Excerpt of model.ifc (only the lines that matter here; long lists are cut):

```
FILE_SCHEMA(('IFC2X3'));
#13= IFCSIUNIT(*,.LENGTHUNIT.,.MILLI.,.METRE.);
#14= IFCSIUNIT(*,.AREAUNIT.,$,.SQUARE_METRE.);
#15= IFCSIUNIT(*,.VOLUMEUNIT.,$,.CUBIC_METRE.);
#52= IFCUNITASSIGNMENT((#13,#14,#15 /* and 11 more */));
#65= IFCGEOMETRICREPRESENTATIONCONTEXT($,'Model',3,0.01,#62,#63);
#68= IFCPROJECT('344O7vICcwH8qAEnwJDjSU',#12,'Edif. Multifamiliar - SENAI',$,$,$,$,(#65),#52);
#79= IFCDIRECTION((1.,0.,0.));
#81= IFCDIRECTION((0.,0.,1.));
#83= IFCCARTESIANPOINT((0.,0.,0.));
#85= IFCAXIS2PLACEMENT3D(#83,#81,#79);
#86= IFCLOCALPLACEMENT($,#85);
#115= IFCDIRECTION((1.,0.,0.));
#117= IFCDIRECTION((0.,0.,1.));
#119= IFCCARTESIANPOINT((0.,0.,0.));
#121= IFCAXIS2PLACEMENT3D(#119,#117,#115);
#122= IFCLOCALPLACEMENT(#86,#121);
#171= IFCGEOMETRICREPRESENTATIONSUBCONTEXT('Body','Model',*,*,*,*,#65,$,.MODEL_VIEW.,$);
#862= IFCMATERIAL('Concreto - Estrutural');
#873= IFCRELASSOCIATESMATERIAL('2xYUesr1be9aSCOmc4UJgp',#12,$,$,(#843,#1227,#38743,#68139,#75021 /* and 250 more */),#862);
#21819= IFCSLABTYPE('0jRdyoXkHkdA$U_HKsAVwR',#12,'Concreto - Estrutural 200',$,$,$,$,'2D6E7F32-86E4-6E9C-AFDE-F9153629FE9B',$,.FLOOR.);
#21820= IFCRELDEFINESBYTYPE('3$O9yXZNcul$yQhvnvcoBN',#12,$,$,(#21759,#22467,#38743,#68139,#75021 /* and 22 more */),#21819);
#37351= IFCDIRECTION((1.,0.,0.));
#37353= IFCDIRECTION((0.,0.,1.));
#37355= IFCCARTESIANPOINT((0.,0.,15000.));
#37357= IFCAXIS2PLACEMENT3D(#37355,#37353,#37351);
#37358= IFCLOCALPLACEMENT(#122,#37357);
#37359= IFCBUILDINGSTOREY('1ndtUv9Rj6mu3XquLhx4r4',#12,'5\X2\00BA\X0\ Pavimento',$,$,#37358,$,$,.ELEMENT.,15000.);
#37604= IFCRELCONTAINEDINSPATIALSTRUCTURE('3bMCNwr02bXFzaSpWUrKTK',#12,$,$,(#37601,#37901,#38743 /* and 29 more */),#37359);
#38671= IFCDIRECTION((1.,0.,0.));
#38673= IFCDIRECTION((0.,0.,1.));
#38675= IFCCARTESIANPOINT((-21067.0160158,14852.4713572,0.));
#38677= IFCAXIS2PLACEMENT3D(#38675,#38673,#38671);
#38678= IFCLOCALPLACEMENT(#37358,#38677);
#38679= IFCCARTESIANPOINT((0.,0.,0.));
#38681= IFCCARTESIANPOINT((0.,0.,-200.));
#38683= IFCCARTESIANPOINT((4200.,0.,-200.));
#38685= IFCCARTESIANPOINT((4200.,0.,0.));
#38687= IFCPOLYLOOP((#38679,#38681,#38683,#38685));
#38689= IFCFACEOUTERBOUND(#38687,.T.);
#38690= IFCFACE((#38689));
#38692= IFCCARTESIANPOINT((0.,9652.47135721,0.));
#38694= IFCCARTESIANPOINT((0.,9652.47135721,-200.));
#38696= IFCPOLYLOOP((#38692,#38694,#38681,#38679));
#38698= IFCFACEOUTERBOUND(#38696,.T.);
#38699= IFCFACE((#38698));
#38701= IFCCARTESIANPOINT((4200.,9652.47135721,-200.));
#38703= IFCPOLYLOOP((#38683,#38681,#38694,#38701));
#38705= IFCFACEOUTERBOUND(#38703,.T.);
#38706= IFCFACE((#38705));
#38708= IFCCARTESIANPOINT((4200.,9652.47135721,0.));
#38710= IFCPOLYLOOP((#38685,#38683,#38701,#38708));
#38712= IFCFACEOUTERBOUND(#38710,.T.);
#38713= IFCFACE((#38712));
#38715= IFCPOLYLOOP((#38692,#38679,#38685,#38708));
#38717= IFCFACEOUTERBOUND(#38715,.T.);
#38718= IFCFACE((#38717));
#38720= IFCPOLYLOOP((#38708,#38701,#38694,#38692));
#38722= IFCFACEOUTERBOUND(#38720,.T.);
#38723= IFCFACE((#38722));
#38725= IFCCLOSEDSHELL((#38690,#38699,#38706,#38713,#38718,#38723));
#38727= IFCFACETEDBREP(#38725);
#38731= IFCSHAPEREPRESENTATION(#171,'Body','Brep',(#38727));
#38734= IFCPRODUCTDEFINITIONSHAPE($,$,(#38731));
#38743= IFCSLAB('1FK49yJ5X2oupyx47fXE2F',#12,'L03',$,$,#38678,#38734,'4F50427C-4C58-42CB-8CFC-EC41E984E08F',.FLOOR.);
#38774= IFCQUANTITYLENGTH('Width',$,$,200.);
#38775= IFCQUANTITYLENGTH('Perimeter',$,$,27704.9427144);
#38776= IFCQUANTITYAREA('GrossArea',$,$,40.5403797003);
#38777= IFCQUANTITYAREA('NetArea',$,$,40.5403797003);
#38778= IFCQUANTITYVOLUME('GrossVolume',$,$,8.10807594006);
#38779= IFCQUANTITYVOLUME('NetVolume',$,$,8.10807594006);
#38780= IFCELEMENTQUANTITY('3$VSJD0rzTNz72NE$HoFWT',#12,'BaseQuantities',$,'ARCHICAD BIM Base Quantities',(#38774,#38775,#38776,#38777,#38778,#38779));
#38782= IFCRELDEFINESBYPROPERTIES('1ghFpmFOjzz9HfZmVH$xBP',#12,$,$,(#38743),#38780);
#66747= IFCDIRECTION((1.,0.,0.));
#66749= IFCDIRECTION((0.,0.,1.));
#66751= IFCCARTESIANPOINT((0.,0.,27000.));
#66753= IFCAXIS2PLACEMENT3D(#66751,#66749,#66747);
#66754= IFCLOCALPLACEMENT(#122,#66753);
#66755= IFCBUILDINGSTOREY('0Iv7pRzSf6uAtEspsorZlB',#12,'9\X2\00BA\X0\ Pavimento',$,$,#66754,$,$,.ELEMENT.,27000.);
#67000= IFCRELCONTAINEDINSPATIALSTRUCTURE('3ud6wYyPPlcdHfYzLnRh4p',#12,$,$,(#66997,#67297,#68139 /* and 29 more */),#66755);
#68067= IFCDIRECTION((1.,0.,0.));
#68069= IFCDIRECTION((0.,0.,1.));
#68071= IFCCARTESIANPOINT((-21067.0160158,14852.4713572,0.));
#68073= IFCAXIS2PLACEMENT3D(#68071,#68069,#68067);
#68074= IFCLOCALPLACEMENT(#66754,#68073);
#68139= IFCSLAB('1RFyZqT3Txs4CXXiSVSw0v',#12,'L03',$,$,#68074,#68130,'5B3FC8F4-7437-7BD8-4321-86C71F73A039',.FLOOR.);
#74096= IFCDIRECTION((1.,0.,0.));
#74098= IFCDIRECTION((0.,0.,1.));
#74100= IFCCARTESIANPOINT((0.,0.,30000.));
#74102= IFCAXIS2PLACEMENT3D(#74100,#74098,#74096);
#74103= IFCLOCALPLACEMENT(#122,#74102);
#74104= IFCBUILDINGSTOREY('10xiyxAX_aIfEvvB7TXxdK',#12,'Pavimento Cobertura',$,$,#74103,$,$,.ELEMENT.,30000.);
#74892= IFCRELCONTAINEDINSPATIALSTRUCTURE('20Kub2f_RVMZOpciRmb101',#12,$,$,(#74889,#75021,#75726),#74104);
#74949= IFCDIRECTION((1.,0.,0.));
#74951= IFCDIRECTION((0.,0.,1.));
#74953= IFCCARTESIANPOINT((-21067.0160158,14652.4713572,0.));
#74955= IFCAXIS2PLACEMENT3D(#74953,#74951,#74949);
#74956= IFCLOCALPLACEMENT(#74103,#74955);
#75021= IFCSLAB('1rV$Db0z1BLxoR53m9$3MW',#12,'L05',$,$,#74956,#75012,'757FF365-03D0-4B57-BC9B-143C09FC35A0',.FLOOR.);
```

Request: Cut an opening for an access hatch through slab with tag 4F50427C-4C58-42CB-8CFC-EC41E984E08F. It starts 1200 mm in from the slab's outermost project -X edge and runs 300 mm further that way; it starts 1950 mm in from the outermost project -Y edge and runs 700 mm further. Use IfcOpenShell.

```python
import numpy as np
import ifcopenshell
import ifcopenshell.api.feature
import ifcopenshell.api.geometry
import ifcopenshell.api.pset
import ifcopenshell.api.root
import ifcopenshell.geom
import ifcopenshell.util.element
import ifcopenshell.util.placement
import ifcopenshell.util.representation
import ifcopenshell.util.shape
import ifcopenshell.util.unit

model = ifcopenshell.open("model.ifc")
unit_scale = ifcopenshell.util.unit.calculate_unit_scale(model)
area_scale = ifcopenshell.util.unit.calculate_unit_scale(model, "AREAUNIT")
volume_scale = ifcopenshell.util.unit.calculate_unit_scale(model, "VOLUMEUNIT")
settings = ifcopenshell.geom.settings()


def volume(element):
    """Net volume in cubic metres, openings subtracted."""
    shape = ifcopenshell.geom.create_shape(settings, element)
    return ifcopenshell.util.shape.get_volume(shape.geometry)


slab = model.by_guid("1FK49yJ5X2oupyx47fXE2F")
before = volume(slab)

# Extent in the slab's own axes, in metres. The edges named are its -X and -Y sides.
slab_shape = ifcopenshell.geom.create_shape(settings, slab)
vertices = ifcopenshell.util.shape.get_vertices(slab_shape.geometry)
x_min, y_min, bottom = vertices.min(axis=0)
top = vertices[:, 2].max()

opening = ifcopenshell.api.root.create_entity(model, ifc_class="IfcOpeningElement", name="Access hatch opening")
context = ifcopenshell.util.representation.get_context(model, "Model", "Body", "MODEL_VIEW")
width, depth = 0.3, 0.7
outline = [(0.0, 0.0), (width, 0.0), (width, depth), (0.0, depth), (0.0, 0.0)]
# Overshoot both faces by 50 mm so the cut is clean.
shape = ifcopenshell.api.geometry.add_slab_representation(
    model, context=context, depth=top - bottom + 0.1, polyline=outline
)
ifcopenshell.api.geometry.assign_representation(model, product=opening, representation=shape)

matrix = ifcopenshell.util.placement.get_local_placement(slab.ObjectPlacement)
matrix[:, 3] = matrix @ np.append(np.array([x_min + 1.2, y_min + 1.95, bottom - 0.05]) / unit_scale, 1.0)
ifcopenshell.api.geometry.edit_object_placement(model, product=opening, matrix=matrix, is_si=False)
ifcopenshell.api.feature.add_feature(model, feature=opening, element=slab)

after = volume(slab)

# Update the slab's stored quantities.
qto = model.by_id(ifcopenshell.util.element.get_pset(slab, "BaseQuantities", should_inherit=False)["id"])
ifcopenshell.api.pset.edit_qto(model, qto=qto, properties={
    "NetArea": after / (top - bottom) / area_scale,
    "NetVolume": after / volume_scale,
})

print(f"slab volume {before:.3f} -> {after:.3f} m3")

model.write("model_rev.ifc")
```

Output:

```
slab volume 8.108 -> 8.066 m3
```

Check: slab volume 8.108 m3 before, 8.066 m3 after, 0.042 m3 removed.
